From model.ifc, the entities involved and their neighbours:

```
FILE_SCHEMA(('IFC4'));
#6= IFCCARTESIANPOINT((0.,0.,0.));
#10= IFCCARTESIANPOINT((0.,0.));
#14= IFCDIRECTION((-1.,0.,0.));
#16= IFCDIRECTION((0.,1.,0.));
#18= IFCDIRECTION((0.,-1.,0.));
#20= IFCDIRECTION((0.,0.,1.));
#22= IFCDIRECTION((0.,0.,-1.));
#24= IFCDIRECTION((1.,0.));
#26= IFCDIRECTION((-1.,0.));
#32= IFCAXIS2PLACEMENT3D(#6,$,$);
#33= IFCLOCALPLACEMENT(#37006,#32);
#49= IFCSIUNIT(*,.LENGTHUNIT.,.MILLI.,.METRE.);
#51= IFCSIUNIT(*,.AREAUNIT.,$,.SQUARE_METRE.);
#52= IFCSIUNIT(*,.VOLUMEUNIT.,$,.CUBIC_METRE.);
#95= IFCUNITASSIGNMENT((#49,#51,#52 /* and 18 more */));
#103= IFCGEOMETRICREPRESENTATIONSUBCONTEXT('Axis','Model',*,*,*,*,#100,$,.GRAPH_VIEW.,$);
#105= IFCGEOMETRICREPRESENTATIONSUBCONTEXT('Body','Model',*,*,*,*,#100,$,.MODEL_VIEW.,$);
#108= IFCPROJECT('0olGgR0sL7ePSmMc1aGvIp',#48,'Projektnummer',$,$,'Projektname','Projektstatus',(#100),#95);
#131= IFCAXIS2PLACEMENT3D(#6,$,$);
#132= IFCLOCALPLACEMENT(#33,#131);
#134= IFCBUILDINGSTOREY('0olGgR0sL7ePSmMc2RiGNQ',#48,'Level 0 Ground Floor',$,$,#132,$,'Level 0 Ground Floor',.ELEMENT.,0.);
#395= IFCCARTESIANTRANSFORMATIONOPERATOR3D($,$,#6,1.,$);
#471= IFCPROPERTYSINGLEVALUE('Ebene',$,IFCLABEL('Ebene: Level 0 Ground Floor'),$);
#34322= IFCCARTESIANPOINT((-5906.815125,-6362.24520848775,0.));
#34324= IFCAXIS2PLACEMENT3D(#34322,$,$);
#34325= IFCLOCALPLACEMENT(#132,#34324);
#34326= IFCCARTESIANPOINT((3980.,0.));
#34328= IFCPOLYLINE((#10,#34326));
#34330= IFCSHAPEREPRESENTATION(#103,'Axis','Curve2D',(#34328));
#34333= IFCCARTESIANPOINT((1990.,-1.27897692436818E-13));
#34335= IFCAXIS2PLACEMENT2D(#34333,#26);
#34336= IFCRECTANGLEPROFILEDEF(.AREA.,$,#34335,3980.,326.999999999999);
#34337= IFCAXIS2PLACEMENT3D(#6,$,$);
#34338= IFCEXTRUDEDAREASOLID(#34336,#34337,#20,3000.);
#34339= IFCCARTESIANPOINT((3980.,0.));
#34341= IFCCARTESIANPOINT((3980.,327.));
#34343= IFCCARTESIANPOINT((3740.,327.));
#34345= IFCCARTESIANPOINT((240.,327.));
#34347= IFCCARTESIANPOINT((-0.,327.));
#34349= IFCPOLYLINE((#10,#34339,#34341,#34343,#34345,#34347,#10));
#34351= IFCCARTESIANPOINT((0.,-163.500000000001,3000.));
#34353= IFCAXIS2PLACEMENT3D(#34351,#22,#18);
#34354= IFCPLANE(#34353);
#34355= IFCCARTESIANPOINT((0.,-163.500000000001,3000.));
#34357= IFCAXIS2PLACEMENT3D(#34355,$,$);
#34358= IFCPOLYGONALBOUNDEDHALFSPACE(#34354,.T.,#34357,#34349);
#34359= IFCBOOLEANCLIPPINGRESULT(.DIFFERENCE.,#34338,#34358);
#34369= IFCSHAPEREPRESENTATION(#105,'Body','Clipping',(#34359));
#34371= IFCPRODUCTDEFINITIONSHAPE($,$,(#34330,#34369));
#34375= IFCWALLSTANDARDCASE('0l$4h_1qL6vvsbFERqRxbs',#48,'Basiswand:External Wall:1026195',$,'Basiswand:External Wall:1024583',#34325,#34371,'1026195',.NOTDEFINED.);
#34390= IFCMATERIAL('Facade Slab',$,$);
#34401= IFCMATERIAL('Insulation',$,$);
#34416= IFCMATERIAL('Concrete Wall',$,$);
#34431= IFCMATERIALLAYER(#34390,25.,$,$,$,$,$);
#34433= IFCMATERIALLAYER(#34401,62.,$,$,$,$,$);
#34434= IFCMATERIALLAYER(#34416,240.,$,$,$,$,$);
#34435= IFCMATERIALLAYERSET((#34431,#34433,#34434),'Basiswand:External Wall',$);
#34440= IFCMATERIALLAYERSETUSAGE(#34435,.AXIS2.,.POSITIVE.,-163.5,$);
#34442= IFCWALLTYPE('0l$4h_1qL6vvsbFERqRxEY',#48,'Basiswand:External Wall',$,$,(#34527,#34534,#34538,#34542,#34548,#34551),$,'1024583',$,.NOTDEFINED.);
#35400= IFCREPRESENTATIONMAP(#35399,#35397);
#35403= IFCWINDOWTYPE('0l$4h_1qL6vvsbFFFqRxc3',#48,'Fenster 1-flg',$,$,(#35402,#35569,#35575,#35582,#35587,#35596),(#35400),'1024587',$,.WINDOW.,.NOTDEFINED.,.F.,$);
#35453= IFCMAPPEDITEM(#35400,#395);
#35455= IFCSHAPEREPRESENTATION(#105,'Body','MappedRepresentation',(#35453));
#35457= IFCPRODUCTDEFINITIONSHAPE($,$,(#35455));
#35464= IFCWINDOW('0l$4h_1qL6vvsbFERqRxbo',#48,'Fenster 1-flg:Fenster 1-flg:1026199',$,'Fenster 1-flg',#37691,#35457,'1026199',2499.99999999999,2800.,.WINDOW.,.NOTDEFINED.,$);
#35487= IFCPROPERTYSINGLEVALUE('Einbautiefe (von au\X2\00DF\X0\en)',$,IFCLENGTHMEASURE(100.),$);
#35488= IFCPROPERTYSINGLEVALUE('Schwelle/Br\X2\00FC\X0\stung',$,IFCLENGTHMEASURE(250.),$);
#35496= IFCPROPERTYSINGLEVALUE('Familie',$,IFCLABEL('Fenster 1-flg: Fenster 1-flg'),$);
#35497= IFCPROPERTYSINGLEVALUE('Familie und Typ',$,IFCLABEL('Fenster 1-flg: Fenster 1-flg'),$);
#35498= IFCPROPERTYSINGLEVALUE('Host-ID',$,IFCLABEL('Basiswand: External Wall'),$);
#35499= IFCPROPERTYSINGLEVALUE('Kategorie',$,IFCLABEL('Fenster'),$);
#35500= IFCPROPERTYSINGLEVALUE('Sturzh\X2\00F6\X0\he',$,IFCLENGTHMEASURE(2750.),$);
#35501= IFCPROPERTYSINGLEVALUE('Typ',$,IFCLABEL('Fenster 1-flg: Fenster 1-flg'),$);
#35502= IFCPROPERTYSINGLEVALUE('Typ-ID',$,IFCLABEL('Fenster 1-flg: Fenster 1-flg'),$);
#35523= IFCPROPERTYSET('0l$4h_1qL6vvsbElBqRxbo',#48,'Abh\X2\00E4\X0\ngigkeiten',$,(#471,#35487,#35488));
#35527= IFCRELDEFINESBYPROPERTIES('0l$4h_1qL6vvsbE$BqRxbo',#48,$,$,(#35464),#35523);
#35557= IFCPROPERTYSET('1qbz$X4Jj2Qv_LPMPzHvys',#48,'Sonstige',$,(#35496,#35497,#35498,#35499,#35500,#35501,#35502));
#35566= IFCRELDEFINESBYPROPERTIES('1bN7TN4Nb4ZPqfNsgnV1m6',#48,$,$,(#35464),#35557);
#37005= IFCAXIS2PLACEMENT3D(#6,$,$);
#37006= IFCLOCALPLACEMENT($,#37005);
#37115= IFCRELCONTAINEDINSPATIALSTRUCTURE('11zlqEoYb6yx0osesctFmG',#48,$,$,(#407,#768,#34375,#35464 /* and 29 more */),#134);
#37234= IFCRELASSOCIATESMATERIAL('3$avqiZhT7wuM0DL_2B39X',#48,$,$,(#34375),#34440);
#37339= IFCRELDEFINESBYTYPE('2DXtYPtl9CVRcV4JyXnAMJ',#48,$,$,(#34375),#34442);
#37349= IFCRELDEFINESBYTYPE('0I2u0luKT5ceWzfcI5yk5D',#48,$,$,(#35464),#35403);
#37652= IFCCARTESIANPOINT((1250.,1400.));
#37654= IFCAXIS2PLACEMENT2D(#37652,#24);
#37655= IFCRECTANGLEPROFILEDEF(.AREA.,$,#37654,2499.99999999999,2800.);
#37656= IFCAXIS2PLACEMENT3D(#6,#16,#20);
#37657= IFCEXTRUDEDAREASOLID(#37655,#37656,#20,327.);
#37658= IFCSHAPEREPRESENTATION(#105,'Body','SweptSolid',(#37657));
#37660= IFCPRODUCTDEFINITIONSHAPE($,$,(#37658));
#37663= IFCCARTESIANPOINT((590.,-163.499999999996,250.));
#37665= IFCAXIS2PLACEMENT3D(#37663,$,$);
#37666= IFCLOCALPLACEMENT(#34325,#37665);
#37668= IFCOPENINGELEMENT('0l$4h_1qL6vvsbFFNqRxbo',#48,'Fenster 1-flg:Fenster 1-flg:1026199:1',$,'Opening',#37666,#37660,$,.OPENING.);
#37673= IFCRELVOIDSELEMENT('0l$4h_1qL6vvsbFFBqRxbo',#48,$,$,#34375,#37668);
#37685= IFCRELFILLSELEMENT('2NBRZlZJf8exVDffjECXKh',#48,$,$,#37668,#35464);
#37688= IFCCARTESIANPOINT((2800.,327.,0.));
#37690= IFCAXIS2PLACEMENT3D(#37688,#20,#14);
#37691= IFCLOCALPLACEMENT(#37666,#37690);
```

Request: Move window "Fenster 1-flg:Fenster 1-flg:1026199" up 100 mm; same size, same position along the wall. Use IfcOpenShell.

```python
import numpy as np
import ifcopenshell
import ifcopenshell.api.geometry
import ifcopenshell.api.pset
import ifcopenshell.util.element
import ifcopenshell.util.placement
import ifcopenshell.util.unit

model = ifcopenshell.open("model.ifc")
unit_scale = ifcopenshell.util.unit.calculate_unit_scale(model)

window = model.by_guid("0l$4h_1qL6vvsbFERqRxbo")
opening = window.FillsVoids[0].RelatingOpeningElement
dz = 0.1 / unit_scale

shift = np.array([0.0, 0.0, dz])
# The window is placed relative to its opening, so it follows when the opening moves.
matrix = ifcopenshell.util.placement.get_local_placement(opening.ObjectPlacement)
matrix[:3, 3] += shift
ifcopenshell.api.geometry.edit_object_placement(
    model, product=opening, matrix=matrix, is_si=False, should_transform_children=True
)

# Keep the stored heights in step.
pset = model.by_id(ifcopenshell.util.element.get_pset(window, "Abhängigkeiten", should_inherit=False)["id"])
ifcopenshell.api.pset.edit_pset(model, pset=pset, properties={
    "Schwelle/Brüstung": model.create_entity("IfcLengthMeasure", ifcopenshell.util.element.get_pset(window, "Abhängigkeiten", "Schwelle/Brüstung") + dz),
})
pset = model.by_id(ifcopenshell.util.element.get_pset(window, "Sonstige", should_inherit=False)["id"])
ifcopenshell.api.pset.edit_pset(model, pset=pset, properties={
    "Sturzhöhe": model.create_entity("IfcLengthMeasure", ifcopenshell.util.element.get_pset(window, "Sonstige", "Sturzhöhe") + dz),
})

print(f"moved by {dz * unit_scale:+.3f} m")

model.write("model_updated.ifc")
```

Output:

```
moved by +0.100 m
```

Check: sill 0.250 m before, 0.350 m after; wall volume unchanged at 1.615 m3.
